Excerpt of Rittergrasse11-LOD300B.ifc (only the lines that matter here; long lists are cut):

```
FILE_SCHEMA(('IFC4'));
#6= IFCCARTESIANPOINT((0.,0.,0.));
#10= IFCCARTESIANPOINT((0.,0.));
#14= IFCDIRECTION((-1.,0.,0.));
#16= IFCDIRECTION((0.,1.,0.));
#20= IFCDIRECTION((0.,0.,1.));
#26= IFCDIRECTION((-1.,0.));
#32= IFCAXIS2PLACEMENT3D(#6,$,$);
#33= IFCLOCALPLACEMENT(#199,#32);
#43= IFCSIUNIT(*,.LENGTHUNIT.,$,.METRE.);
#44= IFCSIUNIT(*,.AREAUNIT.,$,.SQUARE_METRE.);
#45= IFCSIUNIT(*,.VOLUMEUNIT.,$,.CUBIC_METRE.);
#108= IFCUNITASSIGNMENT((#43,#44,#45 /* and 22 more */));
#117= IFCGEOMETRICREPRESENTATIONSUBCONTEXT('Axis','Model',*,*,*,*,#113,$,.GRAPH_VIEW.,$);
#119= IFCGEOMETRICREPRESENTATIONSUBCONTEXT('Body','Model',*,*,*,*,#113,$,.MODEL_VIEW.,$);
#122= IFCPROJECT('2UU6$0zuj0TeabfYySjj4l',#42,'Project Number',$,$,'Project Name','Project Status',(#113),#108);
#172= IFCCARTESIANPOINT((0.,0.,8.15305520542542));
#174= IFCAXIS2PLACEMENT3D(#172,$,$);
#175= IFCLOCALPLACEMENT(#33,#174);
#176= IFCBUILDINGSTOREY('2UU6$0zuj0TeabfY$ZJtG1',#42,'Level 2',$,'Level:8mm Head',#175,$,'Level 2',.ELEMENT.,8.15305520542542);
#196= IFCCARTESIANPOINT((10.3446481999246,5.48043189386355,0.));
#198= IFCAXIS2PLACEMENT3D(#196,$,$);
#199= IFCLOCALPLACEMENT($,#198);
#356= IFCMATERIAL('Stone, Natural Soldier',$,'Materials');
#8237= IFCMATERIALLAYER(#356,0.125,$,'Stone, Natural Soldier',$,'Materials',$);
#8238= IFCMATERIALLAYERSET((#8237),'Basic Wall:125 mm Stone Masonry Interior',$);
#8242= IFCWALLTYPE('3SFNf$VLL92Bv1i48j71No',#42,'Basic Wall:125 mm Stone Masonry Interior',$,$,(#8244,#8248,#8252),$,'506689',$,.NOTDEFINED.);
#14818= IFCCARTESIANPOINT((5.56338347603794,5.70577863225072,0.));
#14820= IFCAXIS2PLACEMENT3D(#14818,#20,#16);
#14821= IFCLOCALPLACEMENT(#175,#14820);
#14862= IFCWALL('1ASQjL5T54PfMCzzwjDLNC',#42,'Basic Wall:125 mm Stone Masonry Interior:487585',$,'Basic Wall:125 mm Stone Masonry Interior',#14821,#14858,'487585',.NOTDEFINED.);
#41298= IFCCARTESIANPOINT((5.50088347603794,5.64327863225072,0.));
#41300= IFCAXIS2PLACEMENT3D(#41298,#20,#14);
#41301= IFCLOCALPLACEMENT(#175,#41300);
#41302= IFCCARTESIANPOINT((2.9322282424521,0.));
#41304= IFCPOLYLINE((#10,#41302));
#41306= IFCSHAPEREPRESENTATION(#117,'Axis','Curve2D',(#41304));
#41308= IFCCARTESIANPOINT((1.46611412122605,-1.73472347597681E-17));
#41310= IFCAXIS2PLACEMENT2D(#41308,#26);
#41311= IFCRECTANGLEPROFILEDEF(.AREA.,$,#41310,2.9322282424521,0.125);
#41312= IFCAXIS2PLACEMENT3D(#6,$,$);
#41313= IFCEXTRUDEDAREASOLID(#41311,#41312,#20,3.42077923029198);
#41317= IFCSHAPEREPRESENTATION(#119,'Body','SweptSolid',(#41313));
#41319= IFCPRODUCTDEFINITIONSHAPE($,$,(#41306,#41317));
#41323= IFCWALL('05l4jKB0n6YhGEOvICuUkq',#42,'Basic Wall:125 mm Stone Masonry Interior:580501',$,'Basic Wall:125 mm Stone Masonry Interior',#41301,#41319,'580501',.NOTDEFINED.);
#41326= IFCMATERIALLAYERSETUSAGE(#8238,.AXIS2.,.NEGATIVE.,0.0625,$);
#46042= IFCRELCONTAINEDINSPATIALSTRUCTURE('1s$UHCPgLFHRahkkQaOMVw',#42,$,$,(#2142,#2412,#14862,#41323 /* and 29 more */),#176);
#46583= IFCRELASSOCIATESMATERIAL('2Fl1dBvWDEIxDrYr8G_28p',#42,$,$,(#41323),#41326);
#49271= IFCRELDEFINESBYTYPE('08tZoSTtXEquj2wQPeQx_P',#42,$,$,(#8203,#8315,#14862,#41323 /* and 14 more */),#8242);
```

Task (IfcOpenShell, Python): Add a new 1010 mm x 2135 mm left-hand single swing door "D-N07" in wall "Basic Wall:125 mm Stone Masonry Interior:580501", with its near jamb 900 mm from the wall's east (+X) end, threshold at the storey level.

```python
import numpy as np
import ifcopenshell
import ifcopenshell.api.feature
import ifcopenshell.api.geometry
import ifcopenshell.api.root
import ifcopenshell.api.spatial
import ifcopenshell.geom
import ifcopenshell.util.element
import ifcopenshell.util.placement
import ifcopenshell.util.representation
import ifcopenshell.util.shape
import ifcopenshell.util.unit

model = ifcopenshell.open("Rittergrasse11-LOD300B.ifc")
unit_scale = ifcopenshell.util.unit.calculate_unit_scale(model)
settings = ifcopenshell.geom.settings()


def volume(element):
    """Net volume in cubic metres, openings subtracted."""
    shape = ifcopenshell.geom.create_shape(settings, element)
    return ifcopenshell.util.shape.get_volume(shape.geometry)


wall = model.by_guid("05l4jKB0n6YhGEOvICuUkq")
storey = ifcopenshell.util.element.get_container(wall, ifc_class="IfcBuildingStorey")
context = ifcopenshell.util.representation.get_context(model, "Model", "Body", "MODEL_VIEW")
before = volume(wall)

width, height, from_end, sill = 1.01, 2.135, 0.9, 0.0  # metres

# The wall runs along its own X axis, and the end named is its -X end.
wall_shape = ifcopenshell.geom.create_shape(settings, wall)
x, y, z = ifcopenshell.util.shape.get_vertices(wall_shape.geometry).T
start = x.min() + from_end
face, thickness = float(y.min()), float(y.max() - y.min())
wall_matrix = ifcopenshell.util.placement.get_local_placement(wall.ObjectPlacement)
level = ifcopenshell.util.placement.get_local_placement(storey.ObjectPlacement)[2, 3]


def in_wall(x, y):
    """Placement at x, y metres in the wall's axes, at sill height."""
    matrix = wall_matrix.copy()
    matrix[:, 3] = wall_matrix @ np.array([x / unit_scale, y / unit_scale, 0.0, 1.0])
    matrix[2, 3] = level + sill / unit_scale
    return matrix


# Opening: a box that overshoots both wall faces by 50 mm.
opening = ifcopenshell.api.root.create_entity(model, ifc_class="IfcOpeningElement", predefined_type="OPENING")
box = ifcopenshell.api.geometry.add_wall_representation(
    model, context=context, length=width, height=height, thickness=thickness + 0.1
)
ifcopenshell.api.geometry.assign_representation(model, product=opening, representation=box)
ifcopenshell.api.geometry.edit_object_placement(model, product=opening, matrix=in_wall(start, face - 0.05), is_si=False)
ifcopenshell.api.feature.add_feature(model, feature=opening, element=wall)

door = ifcopenshell.api.root.create_entity(model, ifc_class="IfcDoor", name="D-N07", predefined_type="DOOR")
door.OverallWidth, door.OverallHeight = width / unit_scale, height / unit_scale
door.OperationType = "SINGLE_SWING_LEFT"
body = ifcopenshell.api.geometry.add_door_representation(
    model,
    context=context,
    overall_width=door.OverallWidth,
    overall_height=door.OverallHeight,
    operation_type="SINGLE_SWING_LEFT",
    lining_properties={"LiningDepth": thickness / unit_scale, "ThresholdDepth": thickness / unit_scale},
)
ifcopenshell.api.geometry.assign_representation(model, product=door, representation=body)
ifcopenshell.api.spatial.assign_container(model, products=[door], relating_structure=storey)
ifcopenshell.api.feature.add_filling(model, opening=opening, element=door)

# The lining spans the wall, so the door starts at the wall face.
ifcopenshell.api.geometry.edit_object_placement(model, product=door, matrix=in_wall(start, face), is_si=False)

after = volume(wall)

print(f"wall volume {before:.3f} -> {after:.3f} m3")

model.write("Rittergrasse11-LOD300B_rev.ifc")
```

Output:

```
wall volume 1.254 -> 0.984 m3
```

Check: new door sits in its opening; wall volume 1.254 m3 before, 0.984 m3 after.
